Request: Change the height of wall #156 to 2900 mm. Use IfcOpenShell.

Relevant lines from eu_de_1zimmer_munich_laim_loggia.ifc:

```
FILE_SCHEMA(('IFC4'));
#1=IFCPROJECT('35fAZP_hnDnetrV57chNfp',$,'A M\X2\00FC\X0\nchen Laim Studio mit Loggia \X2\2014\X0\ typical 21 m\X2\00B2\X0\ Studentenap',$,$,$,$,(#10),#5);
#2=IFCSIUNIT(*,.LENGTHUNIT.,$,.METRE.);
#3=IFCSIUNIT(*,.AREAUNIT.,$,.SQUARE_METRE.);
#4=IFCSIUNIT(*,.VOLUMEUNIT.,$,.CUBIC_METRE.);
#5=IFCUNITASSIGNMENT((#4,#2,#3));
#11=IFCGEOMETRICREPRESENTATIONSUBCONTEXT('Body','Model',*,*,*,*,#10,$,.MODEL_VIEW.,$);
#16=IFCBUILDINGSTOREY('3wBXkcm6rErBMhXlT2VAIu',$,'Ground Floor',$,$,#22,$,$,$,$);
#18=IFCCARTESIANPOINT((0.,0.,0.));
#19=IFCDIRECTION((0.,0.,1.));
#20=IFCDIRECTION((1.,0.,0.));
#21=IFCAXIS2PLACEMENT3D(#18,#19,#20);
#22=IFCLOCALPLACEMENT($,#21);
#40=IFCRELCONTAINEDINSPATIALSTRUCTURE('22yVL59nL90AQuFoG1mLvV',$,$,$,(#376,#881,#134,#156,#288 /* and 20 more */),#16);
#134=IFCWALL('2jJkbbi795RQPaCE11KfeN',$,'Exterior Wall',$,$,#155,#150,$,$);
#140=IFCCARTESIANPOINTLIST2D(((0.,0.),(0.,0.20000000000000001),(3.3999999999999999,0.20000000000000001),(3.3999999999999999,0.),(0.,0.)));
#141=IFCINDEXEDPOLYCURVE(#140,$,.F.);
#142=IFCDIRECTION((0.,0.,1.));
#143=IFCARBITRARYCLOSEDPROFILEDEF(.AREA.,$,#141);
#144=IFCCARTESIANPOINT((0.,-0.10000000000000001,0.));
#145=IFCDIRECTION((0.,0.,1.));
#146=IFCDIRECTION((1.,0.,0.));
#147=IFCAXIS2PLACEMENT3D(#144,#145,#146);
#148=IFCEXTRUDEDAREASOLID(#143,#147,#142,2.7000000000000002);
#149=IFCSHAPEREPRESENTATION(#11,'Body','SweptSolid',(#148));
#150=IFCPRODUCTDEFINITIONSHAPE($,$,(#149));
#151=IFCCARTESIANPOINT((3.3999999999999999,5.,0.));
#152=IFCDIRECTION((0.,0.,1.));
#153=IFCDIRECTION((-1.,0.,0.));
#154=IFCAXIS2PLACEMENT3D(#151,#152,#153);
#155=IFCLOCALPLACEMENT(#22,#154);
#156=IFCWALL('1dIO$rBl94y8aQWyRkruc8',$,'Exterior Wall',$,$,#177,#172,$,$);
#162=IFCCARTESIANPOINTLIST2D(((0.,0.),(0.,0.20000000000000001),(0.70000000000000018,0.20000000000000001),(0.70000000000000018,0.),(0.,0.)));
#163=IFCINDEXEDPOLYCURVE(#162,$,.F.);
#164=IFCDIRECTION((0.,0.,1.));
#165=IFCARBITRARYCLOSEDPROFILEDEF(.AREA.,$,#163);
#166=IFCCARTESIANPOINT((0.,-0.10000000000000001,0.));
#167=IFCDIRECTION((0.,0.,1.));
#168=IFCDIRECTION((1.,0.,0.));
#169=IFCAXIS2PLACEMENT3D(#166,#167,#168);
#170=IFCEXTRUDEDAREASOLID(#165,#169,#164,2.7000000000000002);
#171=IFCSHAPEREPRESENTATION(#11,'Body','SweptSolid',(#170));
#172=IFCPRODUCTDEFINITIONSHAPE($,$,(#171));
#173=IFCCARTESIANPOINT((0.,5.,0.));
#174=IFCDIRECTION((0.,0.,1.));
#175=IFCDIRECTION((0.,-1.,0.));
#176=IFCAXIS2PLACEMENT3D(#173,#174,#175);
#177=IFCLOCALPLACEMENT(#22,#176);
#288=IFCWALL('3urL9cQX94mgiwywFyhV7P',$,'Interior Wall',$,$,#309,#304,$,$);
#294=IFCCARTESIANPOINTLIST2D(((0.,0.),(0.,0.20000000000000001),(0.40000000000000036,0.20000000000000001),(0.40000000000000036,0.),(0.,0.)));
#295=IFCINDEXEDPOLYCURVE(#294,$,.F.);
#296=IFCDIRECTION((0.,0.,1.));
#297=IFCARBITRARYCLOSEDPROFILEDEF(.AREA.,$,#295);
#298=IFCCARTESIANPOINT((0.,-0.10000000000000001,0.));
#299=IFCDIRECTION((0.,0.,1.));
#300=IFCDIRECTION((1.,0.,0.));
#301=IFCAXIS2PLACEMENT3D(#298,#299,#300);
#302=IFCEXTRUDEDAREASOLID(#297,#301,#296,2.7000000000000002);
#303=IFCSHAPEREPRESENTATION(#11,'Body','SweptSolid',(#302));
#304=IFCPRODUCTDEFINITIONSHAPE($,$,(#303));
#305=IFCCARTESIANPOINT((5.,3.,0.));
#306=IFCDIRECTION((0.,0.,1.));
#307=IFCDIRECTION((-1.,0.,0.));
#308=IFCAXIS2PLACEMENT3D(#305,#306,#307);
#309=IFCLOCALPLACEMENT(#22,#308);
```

```python
import ifcopenshell
import ifcopenshell.geom
import ifcopenshell.util.representation
import ifcopenshell.util.shape
import ifcopenshell.util.unit

model = ifcopenshell.open("eu_de_1zimmer_munich_laim_loggia.ifc")
unit_scale = ifcopenshell.util.unit.calculate_unit_scale(model)
settings = ifcopenshell.geom.settings()


def volume(element):
    """Net volume in cubic metres, openings subtracted."""
    shape = ifcopenshell.geom.create_shape(settings, element)
    return ifcopenshell.util.shape.get_volume(shape.geometry)


wall = model.by_guid("1dIO$rBl94y8aQWyRkruc8")
before = volume(wall)

body = ifcopenshell.util.representation.get_representation(wall, "Model", "Body")
solid = body.Items[0]
old_height = solid.Depth
solid.Depth = 2.9 / unit_scale
after = volume(wall)

print(f"height {old_height:g} -> {solid.Depth:g}, volume {before:.3f} -> {after:.3f} m3")

model.write("eu_de_1zimmer_munich_laim_loggia_v2.ifc")
```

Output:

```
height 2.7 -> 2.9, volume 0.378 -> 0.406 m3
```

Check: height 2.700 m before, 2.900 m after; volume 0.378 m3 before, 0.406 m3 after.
